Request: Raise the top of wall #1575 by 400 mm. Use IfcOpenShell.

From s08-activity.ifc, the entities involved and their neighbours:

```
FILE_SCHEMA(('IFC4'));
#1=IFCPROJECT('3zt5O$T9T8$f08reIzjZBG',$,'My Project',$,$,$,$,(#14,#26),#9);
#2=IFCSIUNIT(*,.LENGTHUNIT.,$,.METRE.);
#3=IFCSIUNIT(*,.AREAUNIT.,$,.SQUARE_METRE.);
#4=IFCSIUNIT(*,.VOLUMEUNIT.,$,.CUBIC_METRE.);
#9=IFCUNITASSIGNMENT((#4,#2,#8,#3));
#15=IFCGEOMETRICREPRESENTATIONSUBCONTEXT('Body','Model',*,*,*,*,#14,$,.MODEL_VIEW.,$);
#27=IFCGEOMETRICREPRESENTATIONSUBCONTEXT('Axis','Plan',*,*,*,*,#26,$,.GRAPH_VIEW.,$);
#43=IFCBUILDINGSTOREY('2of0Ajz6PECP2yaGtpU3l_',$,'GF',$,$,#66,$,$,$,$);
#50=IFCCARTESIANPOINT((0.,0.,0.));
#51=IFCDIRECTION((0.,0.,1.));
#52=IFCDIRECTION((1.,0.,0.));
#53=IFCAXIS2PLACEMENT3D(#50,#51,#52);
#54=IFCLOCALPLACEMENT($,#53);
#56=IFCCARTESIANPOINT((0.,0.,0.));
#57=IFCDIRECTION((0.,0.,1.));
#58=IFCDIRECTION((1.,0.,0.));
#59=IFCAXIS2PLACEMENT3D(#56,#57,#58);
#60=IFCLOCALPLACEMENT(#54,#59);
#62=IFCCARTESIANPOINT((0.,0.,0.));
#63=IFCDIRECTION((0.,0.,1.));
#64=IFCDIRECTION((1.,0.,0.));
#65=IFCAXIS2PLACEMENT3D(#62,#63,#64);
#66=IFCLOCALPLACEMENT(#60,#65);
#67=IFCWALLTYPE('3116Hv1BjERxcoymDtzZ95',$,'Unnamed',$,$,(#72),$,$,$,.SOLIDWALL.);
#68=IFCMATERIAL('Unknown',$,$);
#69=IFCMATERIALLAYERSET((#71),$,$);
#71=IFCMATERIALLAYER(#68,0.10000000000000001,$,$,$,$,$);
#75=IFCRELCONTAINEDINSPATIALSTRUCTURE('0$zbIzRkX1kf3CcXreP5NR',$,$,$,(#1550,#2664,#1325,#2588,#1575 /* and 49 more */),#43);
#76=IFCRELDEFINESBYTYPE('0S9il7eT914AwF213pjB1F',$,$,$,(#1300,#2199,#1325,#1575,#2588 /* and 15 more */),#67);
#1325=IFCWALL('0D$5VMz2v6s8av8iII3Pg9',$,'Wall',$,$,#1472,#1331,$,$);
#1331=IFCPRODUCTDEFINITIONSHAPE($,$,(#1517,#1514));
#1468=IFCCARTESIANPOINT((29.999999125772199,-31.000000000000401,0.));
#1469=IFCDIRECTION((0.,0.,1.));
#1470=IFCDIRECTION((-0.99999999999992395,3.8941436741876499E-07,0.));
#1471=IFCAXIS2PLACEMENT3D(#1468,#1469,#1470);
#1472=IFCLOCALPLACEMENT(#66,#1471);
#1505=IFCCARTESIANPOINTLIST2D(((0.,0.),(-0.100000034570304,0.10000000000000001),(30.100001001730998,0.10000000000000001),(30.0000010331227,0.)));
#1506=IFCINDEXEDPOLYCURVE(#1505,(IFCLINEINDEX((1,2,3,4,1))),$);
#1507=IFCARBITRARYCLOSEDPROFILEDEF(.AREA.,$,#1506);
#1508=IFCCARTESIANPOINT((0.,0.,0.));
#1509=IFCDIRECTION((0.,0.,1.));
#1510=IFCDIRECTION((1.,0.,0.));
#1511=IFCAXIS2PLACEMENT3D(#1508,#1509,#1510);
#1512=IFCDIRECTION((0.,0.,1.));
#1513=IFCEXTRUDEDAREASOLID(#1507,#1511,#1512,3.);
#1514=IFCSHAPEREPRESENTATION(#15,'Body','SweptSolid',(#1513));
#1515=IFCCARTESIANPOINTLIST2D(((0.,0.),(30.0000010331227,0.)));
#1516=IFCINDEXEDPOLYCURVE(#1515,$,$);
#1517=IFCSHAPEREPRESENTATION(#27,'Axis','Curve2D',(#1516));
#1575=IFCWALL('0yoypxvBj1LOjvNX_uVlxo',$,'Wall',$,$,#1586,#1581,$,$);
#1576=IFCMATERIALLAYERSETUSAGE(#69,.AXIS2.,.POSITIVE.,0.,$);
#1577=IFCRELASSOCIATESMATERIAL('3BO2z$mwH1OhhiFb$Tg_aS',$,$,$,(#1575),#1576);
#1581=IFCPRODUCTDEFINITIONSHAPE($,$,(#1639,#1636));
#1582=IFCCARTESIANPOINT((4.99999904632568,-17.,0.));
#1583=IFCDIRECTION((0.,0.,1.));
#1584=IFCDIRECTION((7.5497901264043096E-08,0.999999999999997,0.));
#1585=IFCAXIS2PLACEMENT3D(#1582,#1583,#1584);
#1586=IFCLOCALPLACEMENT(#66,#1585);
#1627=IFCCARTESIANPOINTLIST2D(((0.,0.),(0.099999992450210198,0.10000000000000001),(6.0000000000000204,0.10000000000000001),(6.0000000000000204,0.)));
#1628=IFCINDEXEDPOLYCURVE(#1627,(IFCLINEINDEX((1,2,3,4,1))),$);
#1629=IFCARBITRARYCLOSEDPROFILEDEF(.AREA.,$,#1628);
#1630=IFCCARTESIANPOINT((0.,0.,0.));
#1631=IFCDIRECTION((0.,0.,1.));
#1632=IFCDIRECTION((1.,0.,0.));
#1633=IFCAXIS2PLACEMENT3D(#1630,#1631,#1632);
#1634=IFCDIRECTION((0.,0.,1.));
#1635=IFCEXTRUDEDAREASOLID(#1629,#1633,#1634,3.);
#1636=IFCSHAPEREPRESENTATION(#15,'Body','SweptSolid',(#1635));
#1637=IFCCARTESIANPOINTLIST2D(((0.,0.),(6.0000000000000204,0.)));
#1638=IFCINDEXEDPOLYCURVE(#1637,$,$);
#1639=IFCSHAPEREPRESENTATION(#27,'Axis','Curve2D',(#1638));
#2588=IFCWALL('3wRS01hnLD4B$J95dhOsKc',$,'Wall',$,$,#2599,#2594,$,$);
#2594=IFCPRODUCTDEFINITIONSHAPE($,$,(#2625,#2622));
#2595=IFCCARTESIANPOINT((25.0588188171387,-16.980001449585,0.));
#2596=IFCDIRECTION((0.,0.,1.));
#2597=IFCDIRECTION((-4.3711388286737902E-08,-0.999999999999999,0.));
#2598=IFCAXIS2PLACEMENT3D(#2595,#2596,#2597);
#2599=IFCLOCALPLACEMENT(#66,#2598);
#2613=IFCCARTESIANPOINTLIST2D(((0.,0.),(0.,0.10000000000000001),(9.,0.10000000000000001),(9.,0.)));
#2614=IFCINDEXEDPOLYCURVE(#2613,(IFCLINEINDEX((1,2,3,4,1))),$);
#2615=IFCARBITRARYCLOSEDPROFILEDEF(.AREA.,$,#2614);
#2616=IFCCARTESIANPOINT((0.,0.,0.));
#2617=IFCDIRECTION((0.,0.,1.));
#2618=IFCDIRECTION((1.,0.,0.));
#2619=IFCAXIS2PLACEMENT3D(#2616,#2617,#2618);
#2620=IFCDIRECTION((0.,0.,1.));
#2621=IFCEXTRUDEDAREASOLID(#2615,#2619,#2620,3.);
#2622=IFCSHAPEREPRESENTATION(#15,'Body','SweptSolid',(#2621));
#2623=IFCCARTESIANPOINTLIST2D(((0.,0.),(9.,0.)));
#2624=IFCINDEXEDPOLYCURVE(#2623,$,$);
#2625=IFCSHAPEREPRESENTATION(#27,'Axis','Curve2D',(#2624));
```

```python
import ifcopenshell
import ifcopenshell.geom
import ifcopenshell.util.representation
import ifcopenshell.util.shape
import ifcopenshell.util.unit

model = ifcopenshell.open("s08-activity.ifc")
unit_scale = ifcopenshell.util.unit.calculate_unit_scale(model)
settings = ifcopenshell.geom.settings()


def volume(element):
    """Net volume in cubic metres, openings subtracted."""
    shape = ifcopenshell.geom.create_shape(settings, element)
    return ifcopenshell.util.shape.get_volume(shape.geometry)


wall = model.by_id(1575)
before = volume(wall)

body = ifcopenshell.util.representation.get_representation(wall, "Model", "Body")
solid = body.Items[0]
old_height = solid.Depth
solid.Depth += 0.4 / unit_scale
after = volume(wall)

print(f"height {old_height:g} -> {solid.Depth:g}, volume {before:.3f} -> {after:.3f} m3")

model.write("s08-activity_v2.ifc")
```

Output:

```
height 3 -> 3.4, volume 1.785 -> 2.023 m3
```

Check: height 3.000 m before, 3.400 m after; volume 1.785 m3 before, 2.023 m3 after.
